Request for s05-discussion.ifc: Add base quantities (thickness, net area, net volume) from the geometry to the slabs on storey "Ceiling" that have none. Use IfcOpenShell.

First a look at what the model holds.

```python
import ifcopenshell
import ifcopenshell.util.element
import ifcopenshell.util.unit

model = ifcopenshell.open("s05-discussion.ifc")
print(model.schema)
for unit_type in ("LENGTHUNIT", "AREAUNIT", "VOLUMEUNIT"):
    print(unit_type, ifcopenshell.util.unit.calculate_unit_scale(model, unit_type))
storey = next(s for s in model.by_type("IfcBuildingStorey") if s.Name == "Ceiling")
slabs = [e for e in ifcopenshell.util.element.get_decomposition(storey) if e.is_a("IfcSlab")]
for e in sorted(slabs, key=lambda e: e.id()):
    print(e.id(), e.is_a(), e.Name, list(ifcopenshell.util.element.get_psets(e, qtos_only=True)), sep=" | ")
```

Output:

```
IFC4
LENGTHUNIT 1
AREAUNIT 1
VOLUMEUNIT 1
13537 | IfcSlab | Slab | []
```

```python
import ifcopenshell
import ifcopenshell.api.pset
import ifcopenshell.geom
import ifcopenshell.util.element
import ifcopenshell.util.shape
import ifcopenshell.util.unit

model = ifcopenshell.open("s05-discussion.ifc")
unit_scale = ifcopenshell.util.unit.calculate_unit_scale(model)
area_scale = ifcopenshell.util.unit.calculate_unit_scale(model, "AREAUNIT")
volume_scale = ifcopenshell.util.unit.calculate_unit_scale(model, "VOLUMEUNIT")
settings = ifcopenshell.geom.settings()

storey = next(s for s in model.by_type("IfcBuildingStorey") if s.Name == "Ceiling")
slabs = [e for e in ifcopenshell.util.element.get_decomposition(storey) if e.is_a("IfcSlab")]

for e in sorted(slabs, key=lambda e: e.id()):
    if ifcopenshell.util.element.get_psets(e, qtos_only=True, should_inherit=False):
        continue
    # Geometry comes back in metres, in the element's own axes.
    shape = ifcopenshell.geom.create_shape(settings, e)
    values = {
        "Width": ifcopenshell.util.shape.get_z(shape.geometry) / unit_scale,
        "NetArea": ifcopenshell.util.shape.get_footprint_area(shape.geometry) / area_scale,
        "NetVolume": ifcopenshell.util.shape.get_volume(shape.geometry) / volume_scale,
    }
    qto = ifcopenshell.api.pset.add_qto(model, product=e, name="Qto_SlabBaseQuantities")
    ifcopenshell.api.pset.edit_qto(model, qto=qto, properties=values)
    print(e.id(), {k: round(v, 3) for k, v in values.items()})

model.write("s05-discussion_rev.ifc")
```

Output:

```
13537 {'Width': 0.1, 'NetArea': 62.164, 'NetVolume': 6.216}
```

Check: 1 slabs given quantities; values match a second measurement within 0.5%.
